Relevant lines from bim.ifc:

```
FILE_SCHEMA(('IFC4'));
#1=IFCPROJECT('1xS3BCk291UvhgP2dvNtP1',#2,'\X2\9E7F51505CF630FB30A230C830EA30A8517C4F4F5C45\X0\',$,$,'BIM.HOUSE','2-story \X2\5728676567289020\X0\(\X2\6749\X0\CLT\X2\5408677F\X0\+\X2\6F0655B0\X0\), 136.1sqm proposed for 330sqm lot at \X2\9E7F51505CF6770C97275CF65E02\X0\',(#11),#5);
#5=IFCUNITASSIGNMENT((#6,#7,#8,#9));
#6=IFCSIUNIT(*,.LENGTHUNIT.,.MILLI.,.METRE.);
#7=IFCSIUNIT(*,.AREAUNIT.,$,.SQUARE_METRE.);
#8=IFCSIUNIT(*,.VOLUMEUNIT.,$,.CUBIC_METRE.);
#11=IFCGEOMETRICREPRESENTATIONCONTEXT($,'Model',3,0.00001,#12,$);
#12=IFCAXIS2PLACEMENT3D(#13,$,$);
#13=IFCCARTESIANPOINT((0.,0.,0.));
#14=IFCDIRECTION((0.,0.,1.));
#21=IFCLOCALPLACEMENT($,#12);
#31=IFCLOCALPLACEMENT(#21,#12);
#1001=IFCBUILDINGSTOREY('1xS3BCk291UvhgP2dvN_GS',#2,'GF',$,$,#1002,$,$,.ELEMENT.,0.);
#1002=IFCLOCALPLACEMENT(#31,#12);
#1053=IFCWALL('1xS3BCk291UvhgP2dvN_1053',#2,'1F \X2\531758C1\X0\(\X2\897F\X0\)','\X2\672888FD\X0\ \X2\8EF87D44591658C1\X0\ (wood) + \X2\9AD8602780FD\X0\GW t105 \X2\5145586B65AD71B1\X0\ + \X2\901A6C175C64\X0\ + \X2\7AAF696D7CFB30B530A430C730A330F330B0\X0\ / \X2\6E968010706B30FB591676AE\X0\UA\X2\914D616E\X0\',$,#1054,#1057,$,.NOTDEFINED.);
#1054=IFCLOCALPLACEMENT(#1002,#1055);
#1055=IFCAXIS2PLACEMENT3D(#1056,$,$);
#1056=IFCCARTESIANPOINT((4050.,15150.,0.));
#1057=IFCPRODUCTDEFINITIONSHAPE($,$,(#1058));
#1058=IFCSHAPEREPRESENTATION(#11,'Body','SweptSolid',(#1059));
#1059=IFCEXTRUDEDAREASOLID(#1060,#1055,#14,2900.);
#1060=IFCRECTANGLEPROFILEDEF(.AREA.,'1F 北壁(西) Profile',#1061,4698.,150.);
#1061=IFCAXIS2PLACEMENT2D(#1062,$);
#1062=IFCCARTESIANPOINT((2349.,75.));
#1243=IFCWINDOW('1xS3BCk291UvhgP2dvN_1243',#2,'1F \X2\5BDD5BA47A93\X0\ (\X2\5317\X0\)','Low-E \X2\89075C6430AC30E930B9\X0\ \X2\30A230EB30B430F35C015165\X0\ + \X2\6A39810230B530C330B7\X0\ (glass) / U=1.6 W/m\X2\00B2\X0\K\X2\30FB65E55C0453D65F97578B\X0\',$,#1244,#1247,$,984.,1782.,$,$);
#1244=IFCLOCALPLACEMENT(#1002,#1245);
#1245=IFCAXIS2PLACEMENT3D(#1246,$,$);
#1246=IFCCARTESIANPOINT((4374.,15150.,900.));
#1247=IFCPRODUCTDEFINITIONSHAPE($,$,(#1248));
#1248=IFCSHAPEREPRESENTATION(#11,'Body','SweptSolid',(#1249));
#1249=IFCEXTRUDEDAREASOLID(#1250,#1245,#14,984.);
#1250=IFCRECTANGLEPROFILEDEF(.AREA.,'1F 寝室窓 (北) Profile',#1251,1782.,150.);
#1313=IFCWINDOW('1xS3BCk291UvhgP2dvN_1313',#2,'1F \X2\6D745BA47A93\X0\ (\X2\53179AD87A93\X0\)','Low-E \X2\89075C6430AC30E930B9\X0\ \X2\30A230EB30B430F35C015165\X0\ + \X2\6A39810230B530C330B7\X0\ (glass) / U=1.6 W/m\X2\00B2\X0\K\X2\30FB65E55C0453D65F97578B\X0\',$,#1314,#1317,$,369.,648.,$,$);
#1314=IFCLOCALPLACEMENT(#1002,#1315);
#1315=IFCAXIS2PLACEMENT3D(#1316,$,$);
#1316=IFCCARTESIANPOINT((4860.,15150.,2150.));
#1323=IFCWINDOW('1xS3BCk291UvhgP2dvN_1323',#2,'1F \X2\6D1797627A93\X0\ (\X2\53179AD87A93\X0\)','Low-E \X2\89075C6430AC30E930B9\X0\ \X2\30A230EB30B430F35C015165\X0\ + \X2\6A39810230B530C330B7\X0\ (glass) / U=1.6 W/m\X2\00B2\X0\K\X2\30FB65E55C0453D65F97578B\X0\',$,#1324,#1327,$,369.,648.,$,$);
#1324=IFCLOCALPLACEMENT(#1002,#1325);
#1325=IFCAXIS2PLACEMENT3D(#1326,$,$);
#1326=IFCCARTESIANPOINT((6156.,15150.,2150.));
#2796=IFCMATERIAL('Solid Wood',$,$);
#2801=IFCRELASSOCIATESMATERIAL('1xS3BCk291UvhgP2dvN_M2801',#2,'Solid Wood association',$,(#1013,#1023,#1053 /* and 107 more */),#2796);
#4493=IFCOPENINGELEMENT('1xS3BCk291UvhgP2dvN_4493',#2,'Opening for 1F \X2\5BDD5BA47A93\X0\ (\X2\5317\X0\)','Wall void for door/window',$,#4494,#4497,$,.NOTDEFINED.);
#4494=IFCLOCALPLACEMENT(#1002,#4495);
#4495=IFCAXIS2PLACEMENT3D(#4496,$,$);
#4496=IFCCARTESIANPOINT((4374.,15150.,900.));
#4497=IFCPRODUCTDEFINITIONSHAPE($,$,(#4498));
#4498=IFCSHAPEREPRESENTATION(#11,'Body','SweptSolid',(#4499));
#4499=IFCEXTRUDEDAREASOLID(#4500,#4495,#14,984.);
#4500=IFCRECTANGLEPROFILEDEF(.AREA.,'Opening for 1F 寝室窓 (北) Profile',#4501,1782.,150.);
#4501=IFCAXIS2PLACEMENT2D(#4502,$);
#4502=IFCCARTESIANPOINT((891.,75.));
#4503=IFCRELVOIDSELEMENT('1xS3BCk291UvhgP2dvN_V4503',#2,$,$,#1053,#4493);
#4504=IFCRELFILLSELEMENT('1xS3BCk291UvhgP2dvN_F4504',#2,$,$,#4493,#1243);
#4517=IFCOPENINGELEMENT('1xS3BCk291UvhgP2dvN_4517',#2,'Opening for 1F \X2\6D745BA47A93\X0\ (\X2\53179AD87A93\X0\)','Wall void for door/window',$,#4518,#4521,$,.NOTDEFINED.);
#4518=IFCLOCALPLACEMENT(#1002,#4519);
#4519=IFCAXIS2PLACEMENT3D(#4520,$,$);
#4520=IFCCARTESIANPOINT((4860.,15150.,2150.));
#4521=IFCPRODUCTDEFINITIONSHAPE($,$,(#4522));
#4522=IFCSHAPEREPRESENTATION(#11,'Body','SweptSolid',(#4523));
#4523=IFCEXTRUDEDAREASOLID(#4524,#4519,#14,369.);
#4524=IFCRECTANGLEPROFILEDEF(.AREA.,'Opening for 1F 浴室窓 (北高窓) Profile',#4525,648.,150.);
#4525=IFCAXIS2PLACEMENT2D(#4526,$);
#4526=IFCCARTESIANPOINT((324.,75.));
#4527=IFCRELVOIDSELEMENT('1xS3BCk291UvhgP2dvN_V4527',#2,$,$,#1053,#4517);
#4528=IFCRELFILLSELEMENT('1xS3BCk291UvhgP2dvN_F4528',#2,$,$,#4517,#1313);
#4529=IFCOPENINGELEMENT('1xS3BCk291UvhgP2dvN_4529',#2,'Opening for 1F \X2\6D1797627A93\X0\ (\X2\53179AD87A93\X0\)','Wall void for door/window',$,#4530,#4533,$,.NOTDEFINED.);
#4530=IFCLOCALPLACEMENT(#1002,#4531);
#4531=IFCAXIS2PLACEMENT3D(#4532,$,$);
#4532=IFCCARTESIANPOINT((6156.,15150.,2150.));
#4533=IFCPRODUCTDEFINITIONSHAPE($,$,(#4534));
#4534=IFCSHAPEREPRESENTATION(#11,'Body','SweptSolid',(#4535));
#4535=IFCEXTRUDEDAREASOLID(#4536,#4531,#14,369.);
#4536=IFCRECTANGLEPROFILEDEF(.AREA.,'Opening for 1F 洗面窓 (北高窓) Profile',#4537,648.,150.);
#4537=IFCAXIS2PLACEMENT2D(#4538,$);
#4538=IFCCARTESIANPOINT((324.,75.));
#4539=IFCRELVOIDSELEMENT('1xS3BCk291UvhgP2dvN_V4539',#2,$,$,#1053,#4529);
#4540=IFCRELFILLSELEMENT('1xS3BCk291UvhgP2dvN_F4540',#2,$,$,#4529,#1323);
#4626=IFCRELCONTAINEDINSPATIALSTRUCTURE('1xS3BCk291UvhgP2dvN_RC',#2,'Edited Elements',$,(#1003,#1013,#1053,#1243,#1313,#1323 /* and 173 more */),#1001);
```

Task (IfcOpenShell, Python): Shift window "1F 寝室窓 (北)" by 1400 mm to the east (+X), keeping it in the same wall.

```python
import ifcopenshell
import ifcopenshell.api.geometry
import ifcopenshell.util.placement

model = ifcopenshell.open("bim.ifc")

window = model.by_guid("1xS3BCk291UvhgP2dvN_1243")
opening = window.FillsVoids[0].RelatingOpeningElement
wall = opening.VoidsElements[0].RelatingBuildingElement

wall_matrix = ifcopenshell.util.placement.get_local_placement(wall.ObjectPlacement)
shift = wall_matrix[:3, 0] * 1400.0
before = ifcopenshell.util.placement.get_local_placement(window.ObjectPlacement)[:3, 3].copy()

# The window is not placed relative to its opening, so move both.
for product in (opening, window):
    matrix = ifcopenshell.util.placement.get_local_placement(product.ObjectPlacement)
    matrix[:3, 3] += shift
    ifcopenshell.api.geometry.edit_object_placement(model, product=product, matrix=matrix, is_si=False)

after = ifcopenshell.util.placement.get_local_placement(window.ObjectPlacement)[:3, 3]
print("window moved by", (after - before).round(3) + 0.0)

model.write("bim_rev.ifc")
```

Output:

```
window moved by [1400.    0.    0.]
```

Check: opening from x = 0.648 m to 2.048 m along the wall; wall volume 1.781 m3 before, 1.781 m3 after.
